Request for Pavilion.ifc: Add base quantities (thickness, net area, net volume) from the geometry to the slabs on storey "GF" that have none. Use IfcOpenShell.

First a look at what the model holds.

```python
import ifcopenshell
import ifcopenshell.util.element
import ifcopenshell.util.unit

model = ifcopenshell.open("Pavilion.ifc")
print(model.schema)
for unit_type in ("LENGTHUNIT", "AREAUNIT", "VOLUMEUNIT"):
    print(unit_type, ifcopenshell.util.unit.calculate_unit_scale(model, unit_type))
storey = next(s for s in model.by_type("IfcBuildingStorey") if s.Name == "GF")
slabs = [e for e in ifcopenshell.util.element.get_decomposition(storey) if e.is_a("IfcSlab")]
for e in sorted(slabs, key=lambda e: e.id()):
    print(e.id(), e.is_a(), e.Name, list(ifcopenshell.util.element.get_psets(e, qtos_only=True)), sep=" | ")
```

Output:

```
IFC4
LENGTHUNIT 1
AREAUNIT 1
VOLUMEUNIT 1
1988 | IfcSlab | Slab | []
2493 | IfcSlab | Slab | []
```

```python
import ifcopenshell
import ifcopenshell.api.pset
import ifcopenshell.geom
import ifcopenshell.util.element
import ifcopenshell.util.shape
import ifcopenshell.util.unit

model = ifcopenshell.open("Pavilion.ifc")
unit_scale = ifcopenshell.util.unit.calculate_unit_scale(model)
area_scale = ifcopenshell.util.unit.calculate_unit_scale(model, "AREAUNIT")
volume_scale = ifcopenshell.util.unit.calculate_unit_scale(model, "VOLUMEUNIT")
settings = ifcopenshell.geom.settings()

storey = next(s for s in model.by_type("IfcBuildingStorey") if s.Name == "GF")
slabs = [e for e in ifcopenshell.util.element.get_decomposition(storey) if e.is_a("IfcSlab")]

for e in sorted(slabs, key=lambda e: e.id()):
    if ifcopenshell.util.element.get_psets(e, qtos_only=True, should_inherit=False):
        continue
    # Geometry comes back in metres, in the element's own axes.
    shape = ifcopenshell.geom.create_shape(settings, e)
    values = {
        "Width": ifcopenshell.util.shape.get_z(shape.geometry) / unit_scale,
        "NetArea": ifcopenshell.util.shape.get_footprint_area(shape.geometry) / area_scale,
        "NetVolume": ifcopenshell.util.shape.get_volume(shape.geometry) / volume_scale,
    }
    qto = ifcopenshell.api.pset.add_qto(model, product=e, name="Qto_SlabBaseQuantities")
    ifcopenshell.api.pset.edit_qto(model, qto=qto, properties=values)
    print(e.id(), {k: round(v, 3) for k, v in values.items()})

model.write("Pavilion-out.ifc")
```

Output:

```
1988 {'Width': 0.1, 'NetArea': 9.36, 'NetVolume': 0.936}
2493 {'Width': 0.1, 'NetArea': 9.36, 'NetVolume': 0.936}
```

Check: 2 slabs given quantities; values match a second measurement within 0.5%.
